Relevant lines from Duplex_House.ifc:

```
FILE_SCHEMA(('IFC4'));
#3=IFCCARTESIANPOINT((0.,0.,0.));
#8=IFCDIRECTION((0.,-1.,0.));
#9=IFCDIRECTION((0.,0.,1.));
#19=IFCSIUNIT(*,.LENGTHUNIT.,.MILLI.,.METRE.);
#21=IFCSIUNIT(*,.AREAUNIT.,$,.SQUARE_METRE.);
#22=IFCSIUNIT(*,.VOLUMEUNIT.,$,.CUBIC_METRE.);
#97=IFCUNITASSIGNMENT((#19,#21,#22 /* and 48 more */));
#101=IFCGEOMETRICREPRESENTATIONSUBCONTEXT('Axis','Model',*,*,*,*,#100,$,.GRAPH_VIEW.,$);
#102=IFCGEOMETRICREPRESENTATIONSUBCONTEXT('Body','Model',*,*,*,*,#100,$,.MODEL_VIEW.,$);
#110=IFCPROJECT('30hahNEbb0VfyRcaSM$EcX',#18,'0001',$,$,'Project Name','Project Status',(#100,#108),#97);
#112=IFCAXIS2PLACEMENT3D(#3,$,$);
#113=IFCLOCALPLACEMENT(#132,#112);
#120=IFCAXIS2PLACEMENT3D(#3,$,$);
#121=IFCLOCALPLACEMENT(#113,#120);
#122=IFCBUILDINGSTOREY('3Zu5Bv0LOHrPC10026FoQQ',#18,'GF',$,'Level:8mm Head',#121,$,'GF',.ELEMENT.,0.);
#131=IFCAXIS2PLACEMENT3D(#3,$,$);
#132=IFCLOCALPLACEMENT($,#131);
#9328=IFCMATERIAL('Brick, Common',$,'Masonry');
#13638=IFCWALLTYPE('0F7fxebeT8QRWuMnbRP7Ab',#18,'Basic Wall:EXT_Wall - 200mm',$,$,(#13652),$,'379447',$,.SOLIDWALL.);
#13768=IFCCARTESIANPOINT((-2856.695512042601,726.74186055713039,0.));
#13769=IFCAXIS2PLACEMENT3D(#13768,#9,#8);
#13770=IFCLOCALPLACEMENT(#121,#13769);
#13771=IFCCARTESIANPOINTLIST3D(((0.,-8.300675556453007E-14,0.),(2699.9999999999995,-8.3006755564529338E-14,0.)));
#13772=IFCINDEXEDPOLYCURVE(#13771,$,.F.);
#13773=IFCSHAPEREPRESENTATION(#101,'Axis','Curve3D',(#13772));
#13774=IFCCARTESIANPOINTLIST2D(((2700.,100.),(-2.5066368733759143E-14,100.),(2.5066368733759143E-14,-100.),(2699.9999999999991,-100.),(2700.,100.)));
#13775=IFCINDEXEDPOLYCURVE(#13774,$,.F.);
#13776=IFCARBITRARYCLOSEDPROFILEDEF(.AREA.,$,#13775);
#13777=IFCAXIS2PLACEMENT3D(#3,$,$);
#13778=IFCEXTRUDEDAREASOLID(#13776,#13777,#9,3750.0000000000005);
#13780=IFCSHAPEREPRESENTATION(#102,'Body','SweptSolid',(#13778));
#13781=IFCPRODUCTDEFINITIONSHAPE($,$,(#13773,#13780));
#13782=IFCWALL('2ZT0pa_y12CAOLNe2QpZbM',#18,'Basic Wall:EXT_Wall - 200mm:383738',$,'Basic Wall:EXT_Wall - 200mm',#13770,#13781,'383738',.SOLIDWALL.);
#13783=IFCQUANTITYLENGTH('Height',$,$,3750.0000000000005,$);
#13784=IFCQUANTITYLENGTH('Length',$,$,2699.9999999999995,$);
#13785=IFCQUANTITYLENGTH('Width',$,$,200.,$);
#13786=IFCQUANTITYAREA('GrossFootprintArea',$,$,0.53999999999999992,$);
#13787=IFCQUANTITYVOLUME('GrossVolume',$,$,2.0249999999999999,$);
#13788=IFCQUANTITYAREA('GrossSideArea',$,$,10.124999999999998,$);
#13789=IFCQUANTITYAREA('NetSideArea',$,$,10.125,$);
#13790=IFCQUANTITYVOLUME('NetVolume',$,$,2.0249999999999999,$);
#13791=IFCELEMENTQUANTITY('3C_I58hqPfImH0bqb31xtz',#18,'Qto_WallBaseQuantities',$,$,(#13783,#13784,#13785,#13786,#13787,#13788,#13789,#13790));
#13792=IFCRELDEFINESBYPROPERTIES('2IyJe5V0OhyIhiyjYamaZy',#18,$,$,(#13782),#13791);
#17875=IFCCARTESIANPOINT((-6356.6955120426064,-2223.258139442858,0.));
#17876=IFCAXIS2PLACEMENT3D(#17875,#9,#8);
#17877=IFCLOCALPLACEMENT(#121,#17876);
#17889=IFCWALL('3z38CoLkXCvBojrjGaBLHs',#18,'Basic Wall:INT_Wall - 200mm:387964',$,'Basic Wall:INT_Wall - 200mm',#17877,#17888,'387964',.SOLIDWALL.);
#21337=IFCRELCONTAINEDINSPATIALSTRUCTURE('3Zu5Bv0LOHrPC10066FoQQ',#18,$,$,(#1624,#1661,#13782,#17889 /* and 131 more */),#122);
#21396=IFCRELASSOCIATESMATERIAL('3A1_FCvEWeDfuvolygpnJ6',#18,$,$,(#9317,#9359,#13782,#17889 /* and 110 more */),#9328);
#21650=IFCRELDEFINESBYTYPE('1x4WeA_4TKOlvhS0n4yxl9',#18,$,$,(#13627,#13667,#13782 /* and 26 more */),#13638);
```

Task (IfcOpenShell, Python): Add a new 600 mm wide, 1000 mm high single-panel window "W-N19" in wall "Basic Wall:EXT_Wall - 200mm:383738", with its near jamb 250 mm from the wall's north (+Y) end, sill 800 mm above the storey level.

```python
import numpy as np
import ifcopenshell
import ifcopenshell.api.feature
import ifcopenshell.api.geometry
import ifcopenshell.api.pset
import ifcopenshell.api.root
import ifcopenshell.api.spatial
import ifcopenshell.geom
import ifcopenshell.util.element
import ifcopenshell.util.placement
import ifcopenshell.util.representation
import ifcopenshell.util.shape
import ifcopenshell.util.unit

model = ifcopenshell.open("Duplex_House.ifc")
unit_scale = ifcopenshell.util.unit.calculate_unit_scale(model)
area_scale = ifcopenshell.util.unit.calculate_unit_scale(model, "AREAUNIT")
volume_scale = ifcopenshell.util.unit.calculate_unit_scale(model, "VOLUMEUNIT")
settings = ifcopenshell.geom.settings()


def volume(element):
    """Net volume in cubic metres, openings subtracted."""
    shape = ifcopenshell.geom.create_shape(settings, element)
    return ifcopenshell.util.shape.get_volume(shape.geometry)


wall = model.by_guid("2ZT0pa_y12CAOLNe2QpZbM")
storey = ifcopenshell.util.element.get_container(wall, ifc_class="IfcBuildingStorey")
context = ifcopenshell.util.representation.get_context(model, "Model", "Body", "MODEL_VIEW")
before = volume(wall)

width, height, from_end, sill = 0.6, 1, 0.25, 0.8  # metres

# The wall runs along its own X axis, and the end named is its -X end.
wall_shape = ifcopenshell.geom.create_shape(settings, wall)
x, y, z = ifcopenshell.util.shape.get_vertices(wall_shape.geometry).T
start = x.min() + from_end
face, thickness = float(y.min()), float(y.max() - y.min())
wall_matrix = ifcopenshell.util.placement.get_local_placement(wall.ObjectPlacement)
level = ifcopenshell.util.placement.get_local_placement(storey.ObjectPlacement)[2, 3]


def in_wall(x, y):
    """Placement at x, y metres in the wall's axes, at sill height."""
    matrix = wall_matrix.copy()
    matrix[:, 3] = wall_matrix @ np.array([x / unit_scale, y / unit_scale, 0.0, 1.0])
    matrix[2, 3] = level + sill / unit_scale
    return matrix


# Opening: a box that overshoots both wall faces by 50 mm.
opening = ifcopenshell.api.root.create_entity(model, ifc_class="IfcOpeningElement", predefined_type="OPENING")
box = ifcopenshell.api.geometry.add_wall_representation(
    model, context=context, length=width, height=height, thickness=thickness + 0.1
)
ifcopenshell.api.geometry.assign_representation(model, product=opening, representation=box)
ifcopenshell.api.geometry.edit_object_placement(model, product=opening, matrix=in_wall(start, face - 0.05), is_si=False)
ifcopenshell.api.feature.add_feature(model, feature=opening, element=wall)

window = ifcopenshell.api.root.create_entity(model, ifc_class="IfcWindow", name="W-N19", predefined_type="WINDOW")
window.OverallWidth, window.OverallHeight = width / unit_scale, height / unit_scale
window.PartitioningType = "SINGLE_PANEL"
body = ifcopenshell.api.geometry.add_window_representation(
    model,
    context=context,
    overall_width=window.OverallWidth,
    overall_height=window.OverallHeight,
    partition_type="SINGLE_PANEL",
)
ifcopenshell.api.geometry.assign_representation(model, product=window, representation=body)
ifcopenshell.api.spatial.assign_container(model, products=[window], relating_structure=storey)
ifcopenshell.api.feature.add_filling(model, opening=opening, element=window)

# Centre the window in the wall's thickness.
ifcopenshell.api.geometry.edit_object_placement(model, product=window, matrix=in_wall(start, face), is_si=False)
window_shape = ifcopenshell.geom.create_shape(settings, window)
depth = ifcopenshell.util.shape.get_vertices(window_shape.geometry)[:, 1]
offset = face + thickness / 2 - (depth.min() + depth.max()) / 2
ifcopenshell.api.geometry.edit_object_placement(model, product=window, matrix=in_wall(start, offset), is_si=False)

after = volume(wall)

# Update the wall's stored quantities.
qto = model.by_id(ifcopenshell.util.element.get_pset(wall, "Qto_WallBaseQuantities", should_inherit=False)["id"])
ifcopenshell.api.pset.edit_qto(model, qto=qto, properties={
    "NetSideArea": after / thickness / area_scale,
    "NetVolume": after / volume_scale,
})

print(f"wall volume {before:.3f} -> {after:.3f} m3")

model.write("Duplex_House_updated.ifc")
```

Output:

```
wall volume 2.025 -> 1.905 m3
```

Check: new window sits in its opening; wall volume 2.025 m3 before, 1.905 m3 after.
